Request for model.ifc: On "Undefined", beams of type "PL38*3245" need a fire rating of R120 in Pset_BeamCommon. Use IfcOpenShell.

First a look at what the model holds.

```python
import ifcopenshell
import ifcopenshell.util.element

model = ifcopenshell.open("model.ifc")
print(model.schema)
storey = next(s for s in model.by_type("IfcBuildingStorey") if s.Name == "Undefined")
beams = [e for e in ifcopenshell.util.element.get_decomposition(storey) if e.is_a("IfcBeam")]
seen = {}
for e in beams:
    element_type = ifcopenshell.util.element.get_type(e)
    key = (element_type.Name if element_type != e and element_type else None, ifcopenshell.util.element.get_pset(e, "Pset_BeamCommon", "FireRating"))
    seen[key] = seen.get(key, 0) + 1
for (name, value), count in sorted(seen.items(), key=str):
    print(count, "x", name, "|", value)
```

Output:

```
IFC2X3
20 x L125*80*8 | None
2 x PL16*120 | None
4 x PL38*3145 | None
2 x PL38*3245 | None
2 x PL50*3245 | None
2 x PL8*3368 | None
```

```python
import ifcopenshell
import ifcopenshell.api.pset
import ifcopenshell.util.element

model = ifcopenshell.open("model.ifc")

storey = next(s for s in model.by_type("IfcBuildingStorey") if s.Name == "Undefined")
beams = [e for e in ifcopenshell.util.element.get_decomposition(storey) if e.is_a("IfcBeam")]

count = 0
for e in beams:
    element_type = ifcopenshell.util.element.get_type(e)
    if element_type in (None, e) or element_type.Name != "PL38*3245":
        continue
    found = ifcopenshell.util.element.get_pset(e, "Pset_BeamCommon", should_inherit=False)
    if found:
        pset = model.by_id(found["id"])
        if len(ifcopenshell.util.element.get_elements_by_pset(pset)) > 1:
            pset = ifcopenshell.api.pset.unshare_pset(model, products=[e], pset=pset)[0]
    else:
        pset = ifcopenshell.api.pset.add_pset(model, product=e, name="Pset_BeamCommon")
    ifcopenshell.api.pset.edit_pset(model, pset=pset, properties={"FireRating": "R120"})
    count += 1

print(count, "beams updated")

model.write("model-out.ifc")
```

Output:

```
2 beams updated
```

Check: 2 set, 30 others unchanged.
